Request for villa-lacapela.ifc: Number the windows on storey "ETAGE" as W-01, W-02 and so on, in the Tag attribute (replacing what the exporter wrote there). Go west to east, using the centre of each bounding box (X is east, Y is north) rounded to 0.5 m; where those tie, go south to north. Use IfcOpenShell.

First a look at what the model holds.

```python
import ifcopenshell
import ifcopenshell.util.element
import ifcopenshell.util.placement

model = ifcopenshell.open("villa-lacapela.ifc")
print(model.schema)
storey = next(s for s in model.by_type("IfcBuildingStorey") if s.Name == "ETAGE")
windows = [e for e in ifcopenshell.util.element.get_decomposition(storey) if e.is_a("IfcWindow")]
for e in sorted(windows, key=lambda e: e.id()):
    origin = ifcopenshell.util.placement.get_local_placement(e.ObjectPlacement)[:3, 3]
    print(e.id(), e.Tag, e.Name, origin.round(2) + 0.0, sep=" | ")
```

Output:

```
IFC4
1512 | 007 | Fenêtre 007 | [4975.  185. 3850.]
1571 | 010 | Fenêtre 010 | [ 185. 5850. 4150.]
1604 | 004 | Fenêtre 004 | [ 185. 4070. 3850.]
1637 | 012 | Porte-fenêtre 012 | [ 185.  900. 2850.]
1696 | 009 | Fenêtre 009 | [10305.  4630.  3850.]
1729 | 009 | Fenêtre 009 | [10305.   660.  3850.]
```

```python
import ifcopenshell
import ifcopenshell.geom
import ifcopenshell.util.element
import ifcopenshell.util.shape

model = ifcopenshell.open("villa-lacapela.ifc")
settings = ifcopenshell.geom.settings()
settings.set("use-world-coords", True)


def centre(element):
    shape = ifcopenshell.geom.create_shape(settings, element)
    return ifcopenshell.util.shape.get_bbox_centroid(shape.geometry)


storey = next(s for s in model.by_type("IfcBuildingStorey") if s.Name == "ETAGE")
windows = [e for e in ifcopenshell.util.element.get_decomposition(storey) if e.is_a("IfcWindow")]

# Insertion points can sit at a corner or the storey origin, so sort by the geometry (in metres).
centres = {e: centre(e) for e in windows}
windows.sort(key=lambda e: (round(centres[e][0] / 0.5), centres[e][1]))

for i, e in enumerate(windows, start=1):
    number = f"W-{i:02d}"
    e.Tag = number
    print(e.id(), number)

model.write("villa-lacapela-out.ifc")
```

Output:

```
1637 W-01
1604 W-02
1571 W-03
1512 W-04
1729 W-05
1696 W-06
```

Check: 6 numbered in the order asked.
